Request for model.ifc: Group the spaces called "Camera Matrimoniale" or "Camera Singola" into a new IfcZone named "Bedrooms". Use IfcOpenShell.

First a look at what the model holds.

```python
import ifcopenshell

model = ifcopenshell.open("model.ifc")
print(model.schema)
seen = {}
for space in model.by_type("IfcSpace"):
    seen[space.LongName] = seen.get(space.LongName, 0) + 1
for name, count in sorted(seen.items(), key=str):
    print(count, "x", name)
print("zones:", [z.Name for z in model.by_type("IfcZone")][:20])
```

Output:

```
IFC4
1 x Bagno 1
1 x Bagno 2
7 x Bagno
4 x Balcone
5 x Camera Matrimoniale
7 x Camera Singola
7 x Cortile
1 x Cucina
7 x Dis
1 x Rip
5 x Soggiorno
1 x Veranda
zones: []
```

```python
import ifcopenshell
import ifcopenshell.api.group
import ifcopenshell.api.root

model = ifcopenshell.open("model.ifc")

names = {"Camera Matrimoniale", "Camera Singola"}
spaces = [s for s in model.by_type("IfcSpace") if s.LongName in names]

zone = ifcopenshell.api.root.create_entity(model, ifc_class="IfcZone", name="Bedrooms")
ifcopenshell.api.group.assign_group(model, products=spaces, group=zone)
print(len(spaces), "spaces in", zone.Name)

model.write("model_updated.ifc")
```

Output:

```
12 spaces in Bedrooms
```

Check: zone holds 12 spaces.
